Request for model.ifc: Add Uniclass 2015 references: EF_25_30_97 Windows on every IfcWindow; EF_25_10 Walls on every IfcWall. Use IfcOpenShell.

First a look at what the model holds.

```python
import ifcopenshell

model = ifcopenshell.open("model.ifc")
print(model.schema)
print("classifications:", [c.Name for c in model.by_type("IfcClassification")])
for ifc_class in ("IfcDoor", "IfcRoof", "IfcStair", "IfcWall", "IfcWindow"):
    print(ifc_class, len(model.by_type(ifc_class)))
```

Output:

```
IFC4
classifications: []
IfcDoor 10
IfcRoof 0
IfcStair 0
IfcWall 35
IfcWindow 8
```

```python
import ifcopenshell
import ifcopenshell.api.classification

model = ifcopenshell.open("model.ifc")

system = ifcopenshell.api.classification.add_classification(model, classification="Uniclass 2015")

codes = {
    "IfcWindow": ("EF_25_30_97", "Windows"),
    "IfcWall": ("EF_25_10", "Walls"),
}
for ifc_class, (code, name) in codes.items():
    products = model.by_type(ifc_class)
    ifcopenshell.api.classification.add_reference(
        model, products=products, classification=system, identification=code, name=name
    )
    print(code, len(products))

model.write("model_v2.ifc")
```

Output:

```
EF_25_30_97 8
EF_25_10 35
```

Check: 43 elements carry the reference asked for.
